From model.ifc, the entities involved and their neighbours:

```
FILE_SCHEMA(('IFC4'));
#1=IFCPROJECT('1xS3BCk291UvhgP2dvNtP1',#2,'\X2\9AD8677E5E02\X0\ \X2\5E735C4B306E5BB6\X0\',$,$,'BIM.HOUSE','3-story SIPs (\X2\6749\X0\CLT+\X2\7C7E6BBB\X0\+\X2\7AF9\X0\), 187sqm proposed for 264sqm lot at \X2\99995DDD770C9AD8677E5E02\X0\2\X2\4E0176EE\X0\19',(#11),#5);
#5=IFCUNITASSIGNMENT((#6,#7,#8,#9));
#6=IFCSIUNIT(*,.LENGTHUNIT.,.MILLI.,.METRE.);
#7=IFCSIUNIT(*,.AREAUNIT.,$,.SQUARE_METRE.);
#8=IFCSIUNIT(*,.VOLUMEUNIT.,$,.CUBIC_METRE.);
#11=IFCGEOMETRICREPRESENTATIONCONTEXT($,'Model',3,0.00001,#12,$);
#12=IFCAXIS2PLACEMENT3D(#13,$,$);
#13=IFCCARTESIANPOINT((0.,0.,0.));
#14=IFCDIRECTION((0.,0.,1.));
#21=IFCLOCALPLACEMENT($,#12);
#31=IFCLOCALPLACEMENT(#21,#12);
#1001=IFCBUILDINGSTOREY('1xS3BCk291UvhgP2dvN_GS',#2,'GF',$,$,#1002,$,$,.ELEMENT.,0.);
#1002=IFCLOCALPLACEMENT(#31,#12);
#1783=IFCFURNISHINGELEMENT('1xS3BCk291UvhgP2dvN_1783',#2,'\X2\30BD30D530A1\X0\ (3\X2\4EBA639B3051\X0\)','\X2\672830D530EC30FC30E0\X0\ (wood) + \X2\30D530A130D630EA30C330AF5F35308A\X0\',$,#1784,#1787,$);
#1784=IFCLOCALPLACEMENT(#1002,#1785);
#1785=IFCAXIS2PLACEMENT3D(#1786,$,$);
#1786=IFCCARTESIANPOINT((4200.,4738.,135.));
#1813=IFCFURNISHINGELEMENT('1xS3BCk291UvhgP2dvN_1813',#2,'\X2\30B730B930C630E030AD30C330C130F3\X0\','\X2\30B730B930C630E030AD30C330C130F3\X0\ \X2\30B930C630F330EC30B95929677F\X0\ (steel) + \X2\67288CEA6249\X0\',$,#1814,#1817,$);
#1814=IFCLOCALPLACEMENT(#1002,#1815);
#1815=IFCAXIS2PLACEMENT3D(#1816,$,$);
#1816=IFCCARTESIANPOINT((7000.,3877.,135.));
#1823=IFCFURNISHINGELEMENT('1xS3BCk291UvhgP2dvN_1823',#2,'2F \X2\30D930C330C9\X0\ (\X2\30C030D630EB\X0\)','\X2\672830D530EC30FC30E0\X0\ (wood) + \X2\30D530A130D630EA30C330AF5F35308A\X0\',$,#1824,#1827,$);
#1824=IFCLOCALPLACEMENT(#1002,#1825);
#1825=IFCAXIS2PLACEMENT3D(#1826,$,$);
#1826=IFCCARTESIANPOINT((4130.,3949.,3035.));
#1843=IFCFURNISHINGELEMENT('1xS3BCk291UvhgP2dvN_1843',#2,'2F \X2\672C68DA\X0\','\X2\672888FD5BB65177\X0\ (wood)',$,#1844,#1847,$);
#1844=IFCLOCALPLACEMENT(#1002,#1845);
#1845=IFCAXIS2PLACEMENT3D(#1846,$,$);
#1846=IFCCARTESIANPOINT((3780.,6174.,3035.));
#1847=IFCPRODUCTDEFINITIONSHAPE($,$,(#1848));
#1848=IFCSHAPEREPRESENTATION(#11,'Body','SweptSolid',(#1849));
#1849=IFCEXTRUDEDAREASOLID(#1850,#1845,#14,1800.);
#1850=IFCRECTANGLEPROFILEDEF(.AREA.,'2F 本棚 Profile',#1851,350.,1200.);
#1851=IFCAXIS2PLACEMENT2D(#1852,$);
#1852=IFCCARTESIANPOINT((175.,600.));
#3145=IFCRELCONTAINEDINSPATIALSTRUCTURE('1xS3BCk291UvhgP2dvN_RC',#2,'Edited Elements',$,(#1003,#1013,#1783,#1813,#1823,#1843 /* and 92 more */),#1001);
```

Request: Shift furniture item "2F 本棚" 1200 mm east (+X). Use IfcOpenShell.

```python
import ifcopenshell
import ifcopenshell.api.geometry
import ifcopenshell.util.placement
import ifcopenshell.util.unit

model = ifcopenshell.open("model.ifc")
unit_scale = ifcopenshell.util.unit.calculate_unit_scale(model)

item = model.by_guid("1xS3BCk291UvhgP2dvN_1843")
matrix = ifcopenshell.util.placement.get_local_placement(item.ObjectPlacement)
matrix[0, 3] += 1.2 / unit_scale
ifcopenshell.api.geometry.edit_object_placement(model, product=item, matrix=matrix, is_si=False)

print(ifcopenshell.util.placement.get_local_placement(item.ObjectPlacement).round(3) + 0.0)

model.write("model_updated.ifc")
```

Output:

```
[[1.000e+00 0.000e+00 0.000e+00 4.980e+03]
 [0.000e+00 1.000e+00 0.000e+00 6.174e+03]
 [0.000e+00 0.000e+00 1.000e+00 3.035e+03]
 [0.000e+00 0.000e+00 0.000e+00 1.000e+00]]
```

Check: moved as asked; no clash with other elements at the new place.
